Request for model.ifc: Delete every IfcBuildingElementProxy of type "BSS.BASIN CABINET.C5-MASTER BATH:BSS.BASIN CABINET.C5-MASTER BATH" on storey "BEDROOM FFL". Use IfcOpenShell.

First a look at what the model holds.

```python
import ifcopenshell
import ifcopenshell.util.element

model = ifcopenshell.open("model.ifc")
print(model.schema)
storey = next(s for s in model.by_type("IfcBuildingStorey") if s.Name == "BEDROOM FFL")
proxies = [e for e in ifcopenshell.util.element.get_decomposition(storey) if e.is_a("IfcBuildingElementProxy")]
seen = {}
for e in proxies:
    element_type = ifcopenshell.util.element.get_type(e)
    name = element_type.Name if element_type not in (None, e) else None
    seen[name] = seen.get(name, 0) + 1
for name, count in sorted(seen.items(), key=str):
    print(count, "x", name)
```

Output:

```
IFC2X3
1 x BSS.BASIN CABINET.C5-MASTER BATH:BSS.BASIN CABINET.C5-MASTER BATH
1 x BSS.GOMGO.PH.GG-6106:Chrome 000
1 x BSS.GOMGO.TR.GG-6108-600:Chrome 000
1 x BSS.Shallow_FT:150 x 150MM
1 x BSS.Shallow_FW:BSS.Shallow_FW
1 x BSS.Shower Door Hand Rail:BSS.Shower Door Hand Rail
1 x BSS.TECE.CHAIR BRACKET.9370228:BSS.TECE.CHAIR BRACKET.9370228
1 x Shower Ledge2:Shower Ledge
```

```python
import ifcopenshell
import ifcopenshell.api.root
import ifcopenshell.util.element

model = ifcopenshell.open("model.ifc")

storey = next(s for s in model.by_type("IfcBuildingStorey") if s.Name == "BEDROOM FFL")
proxies = [e for e in ifcopenshell.util.element.get_decomposition(storey) if e.is_a("IfcBuildingElementProxy")]
targets = [e for e in proxies if (t := ifcopenshell.util.element.get_type(e)) not in (None, e) and t.Name == "BSS.BASIN CABINET.C5-MASTER BATH:BSS.BASIN CABINET.C5-MASTER BATH"]

for e in targets:
    ifcopenshell.api.root.remove_product(model, product=e)
print(len(targets), "removed")

model.write("model_v2.ifc")
```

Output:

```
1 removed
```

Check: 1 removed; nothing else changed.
